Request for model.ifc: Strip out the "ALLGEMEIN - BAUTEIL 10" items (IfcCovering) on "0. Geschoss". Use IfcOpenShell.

First a look at what the model holds.

```python
import ifcopenshell
import ifcopenshell.util.element

model = ifcopenshell.open("model.ifc")
print(model.schema)
storey = next(s for s in model.by_type("IfcBuildingStorey") if s.Name == "0. Geschoss")
coverings = [e for e in ifcopenshell.util.element.get_decomposition(storey) if e.is_a("IfcCovering")]
seen = {}
for e in coverings:
    element_type = ifcopenshell.util.element.get_type(e)
    name = element_type.Name if element_type not in (None, e) else None
    seen[name] = seen.get(name, 0) + 1
for name, count in sorted(seen.items(), key=str):
    print(count, "x", name)
```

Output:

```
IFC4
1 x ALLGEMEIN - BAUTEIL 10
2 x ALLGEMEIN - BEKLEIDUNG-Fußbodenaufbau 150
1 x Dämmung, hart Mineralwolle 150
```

```python
import ifcopenshell
import ifcopenshell.api.root
import ifcopenshell.util.element

model = ifcopenshell.open("model.ifc")

storey = next(s for s in model.by_type("IfcBuildingStorey") if s.Name == "0. Geschoss")
coverings = [e for e in ifcopenshell.util.element.get_decomposition(storey) if e.is_a("IfcCovering")]
targets = [e for e in coverings if (t := ifcopenshell.util.element.get_type(e)) not in (None, e) and t.Name == "ALLGEMEIN - BAUTEIL 10"]

for e in targets:
    ifcopenshell.api.root.remove_product(model, product=e)
print(len(targets), "removed")

model.write("model_edited.ifc")
```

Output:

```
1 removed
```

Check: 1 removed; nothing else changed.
